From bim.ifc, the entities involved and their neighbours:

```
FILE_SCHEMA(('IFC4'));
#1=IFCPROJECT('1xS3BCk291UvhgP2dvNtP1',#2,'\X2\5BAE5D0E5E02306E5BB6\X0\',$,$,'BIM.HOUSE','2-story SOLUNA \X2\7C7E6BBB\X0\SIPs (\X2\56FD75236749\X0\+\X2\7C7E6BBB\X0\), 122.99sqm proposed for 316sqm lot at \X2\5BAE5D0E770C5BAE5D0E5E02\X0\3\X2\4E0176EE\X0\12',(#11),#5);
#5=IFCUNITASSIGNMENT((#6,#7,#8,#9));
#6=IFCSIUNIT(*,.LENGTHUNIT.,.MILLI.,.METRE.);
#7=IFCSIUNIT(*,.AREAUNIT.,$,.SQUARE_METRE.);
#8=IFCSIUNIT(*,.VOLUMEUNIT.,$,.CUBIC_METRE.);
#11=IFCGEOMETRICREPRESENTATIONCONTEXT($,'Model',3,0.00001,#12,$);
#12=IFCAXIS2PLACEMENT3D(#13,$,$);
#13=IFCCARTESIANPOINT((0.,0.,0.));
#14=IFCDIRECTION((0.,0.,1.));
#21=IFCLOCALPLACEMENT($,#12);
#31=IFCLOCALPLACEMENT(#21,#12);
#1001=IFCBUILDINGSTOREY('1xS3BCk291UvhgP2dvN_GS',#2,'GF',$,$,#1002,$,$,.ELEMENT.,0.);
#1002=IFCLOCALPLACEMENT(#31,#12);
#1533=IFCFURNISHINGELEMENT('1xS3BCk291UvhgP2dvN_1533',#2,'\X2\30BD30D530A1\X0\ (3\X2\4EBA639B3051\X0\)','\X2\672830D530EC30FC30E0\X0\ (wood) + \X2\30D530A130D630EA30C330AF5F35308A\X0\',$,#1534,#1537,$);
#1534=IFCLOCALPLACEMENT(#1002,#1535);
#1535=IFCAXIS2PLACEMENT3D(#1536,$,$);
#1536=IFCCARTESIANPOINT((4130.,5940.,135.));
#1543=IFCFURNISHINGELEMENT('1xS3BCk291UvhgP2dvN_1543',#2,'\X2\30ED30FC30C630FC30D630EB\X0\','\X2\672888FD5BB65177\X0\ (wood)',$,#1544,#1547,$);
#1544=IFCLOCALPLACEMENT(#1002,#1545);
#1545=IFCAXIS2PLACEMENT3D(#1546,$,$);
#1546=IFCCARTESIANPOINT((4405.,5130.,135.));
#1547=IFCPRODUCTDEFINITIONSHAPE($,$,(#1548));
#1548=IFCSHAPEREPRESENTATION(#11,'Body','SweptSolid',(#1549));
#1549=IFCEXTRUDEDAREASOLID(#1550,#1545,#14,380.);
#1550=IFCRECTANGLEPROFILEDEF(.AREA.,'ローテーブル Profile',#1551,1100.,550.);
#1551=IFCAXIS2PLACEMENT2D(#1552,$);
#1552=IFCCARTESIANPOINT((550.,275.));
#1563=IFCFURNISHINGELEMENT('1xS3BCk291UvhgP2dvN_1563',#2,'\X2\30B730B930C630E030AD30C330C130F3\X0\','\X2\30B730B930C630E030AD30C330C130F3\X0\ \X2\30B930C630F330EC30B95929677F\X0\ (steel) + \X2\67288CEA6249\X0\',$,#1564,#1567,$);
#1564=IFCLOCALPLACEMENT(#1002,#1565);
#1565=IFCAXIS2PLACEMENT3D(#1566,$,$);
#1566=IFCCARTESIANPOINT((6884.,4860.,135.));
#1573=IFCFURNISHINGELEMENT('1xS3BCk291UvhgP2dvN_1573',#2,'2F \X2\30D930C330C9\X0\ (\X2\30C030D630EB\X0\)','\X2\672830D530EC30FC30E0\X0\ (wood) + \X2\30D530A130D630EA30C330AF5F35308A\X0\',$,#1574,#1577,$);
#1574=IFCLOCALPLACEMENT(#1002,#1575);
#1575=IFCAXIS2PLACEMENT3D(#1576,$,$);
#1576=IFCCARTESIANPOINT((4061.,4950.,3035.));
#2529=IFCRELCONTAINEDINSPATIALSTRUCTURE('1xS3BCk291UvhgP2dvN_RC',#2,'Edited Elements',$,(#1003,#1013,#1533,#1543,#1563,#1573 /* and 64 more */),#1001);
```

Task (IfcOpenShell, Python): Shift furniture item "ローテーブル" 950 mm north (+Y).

```python
import ifcopenshell
import ifcopenshell.api.geometry
import ifcopenshell.util.placement

model = ifcopenshell.open("bim.ifc")

item = model.by_guid("1xS3BCk291UvhgP2dvN_1543")
matrix = ifcopenshell.util.placement.get_local_placement(item.ObjectPlacement)
matrix[1, 3] += 950.0
ifcopenshell.api.geometry.edit_object_placement(model, product=item, matrix=matrix, is_si=False)

print(ifcopenshell.util.placement.get_local_placement(item.ObjectPlacement).round(3) + 0.0)

model.write("bim_updated.ifc")
```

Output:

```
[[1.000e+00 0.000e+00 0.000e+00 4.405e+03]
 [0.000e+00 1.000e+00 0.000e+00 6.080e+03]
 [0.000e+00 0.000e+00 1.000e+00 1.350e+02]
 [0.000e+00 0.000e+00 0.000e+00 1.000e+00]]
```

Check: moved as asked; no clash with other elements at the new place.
